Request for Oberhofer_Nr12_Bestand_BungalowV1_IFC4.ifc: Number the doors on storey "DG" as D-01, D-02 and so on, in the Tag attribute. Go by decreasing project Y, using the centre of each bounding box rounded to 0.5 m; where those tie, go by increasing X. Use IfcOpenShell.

First a look at what the model holds.

```python
import ifcopenshell
import ifcopenshell.util.element
import ifcopenshell.util.placement

model = ifcopenshell.open("Oberhofer_Nr12_Bestand_BungalowV1_IFC4.ifc")
print(model.schema)
storey = next(s for s in model.by_type("IfcBuildingStorey") if s.Name == "DG")
doors = [e for e in ifcopenshell.util.element.get_decomposition(storey) if e.is_a("IfcDoor")]
for e in sorted(doors, key=lambda e: e.id()):
    origin = ifcopenshell.util.placement.get_local_placement(e.ObjectPlacement)[:3, 3]
    print(e.id(), e.Tag, e.Name, origin.round(2) + 0.0, sep=" | ")
```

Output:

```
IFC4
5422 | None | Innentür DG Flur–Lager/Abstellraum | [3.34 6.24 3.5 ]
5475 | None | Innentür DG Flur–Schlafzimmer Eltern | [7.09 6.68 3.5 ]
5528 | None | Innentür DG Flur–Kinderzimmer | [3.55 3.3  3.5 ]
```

```python
import ifcopenshell
import ifcopenshell.geom
import ifcopenshell.util.element
import ifcopenshell.util.shape

model = ifcopenshell.open("Oberhofer_Nr12_Bestand_BungalowV1_IFC4.ifc")
settings = ifcopenshell.geom.settings()
settings.set("use-world-coords", True)


def centre(element):
    shape = ifcopenshell.geom.create_shape(settings, element)
    return ifcopenshell.util.shape.get_bbox_centroid(shape.geometry)


storey = next(s for s in model.by_type("IfcBuildingStorey") if s.Name == "DG")
doors = [e for e in ifcopenshell.util.element.get_decomposition(storey) if e.is_a("IfcDoor")]

# Insertion points can sit at a corner or the storey origin, so sort by the geometry (in metres).
centres = {e: centre(e) for e in doors}
doors.sort(key=lambda e: (-round(centres[e][1] / 0.5), centres[e][0]))

for i, e in enumerate(doors, start=1):
    number = f"D-{i:02d}"
    e.Tag = number
    print(e.id(), number)

model.write("Oberhofer_Nr12_Bestand_BungalowV1_IFC4_v2.ifc")
```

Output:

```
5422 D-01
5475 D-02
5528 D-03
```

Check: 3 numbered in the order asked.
